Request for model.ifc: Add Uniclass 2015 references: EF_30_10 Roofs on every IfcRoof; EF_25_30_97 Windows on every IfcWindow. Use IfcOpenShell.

First a look at what the model holds.

```python
import ifcopenshell

model = ifcopenshell.open("model.ifc")
print(model.schema)
print("classifications:", [c.Name for c in model.by_type("IfcClassification")])
for ifc_class in ("IfcDoor", "IfcRoof", "IfcStair", "IfcWall", "IfcWindow"):
    print(ifc_class, len(model.by_type(ifc_class)))
```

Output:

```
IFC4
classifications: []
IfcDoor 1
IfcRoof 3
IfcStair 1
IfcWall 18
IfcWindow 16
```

```python
import ifcopenshell
import ifcopenshell.api.classification

model = ifcopenshell.open("model.ifc")

system = ifcopenshell.api.classification.add_classification(model, classification="Uniclass 2015")

codes = {
    "IfcRoof": ("EF_30_10", "Roofs"),
    "IfcWindow": ("EF_25_30_97", "Windows"),
}
for ifc_class, (code, name) in codes.items():
    products = model.by_type(ifc_class)
    ifcopenshell.api.classification.add_reference(
        model, products=products, classification=system, identification=code, name=name
    )
    print(code, len(products))

model.write("model_rev.ifc")
```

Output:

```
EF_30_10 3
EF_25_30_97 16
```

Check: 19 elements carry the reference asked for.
